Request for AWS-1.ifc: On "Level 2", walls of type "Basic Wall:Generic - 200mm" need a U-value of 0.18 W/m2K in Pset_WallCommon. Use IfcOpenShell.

First a look at what the model holds.

```python
import ifcopenshell
import ifcopenshell.util.element

model = ifcopenshell.open("AWS-1.ifc")
print(model.schema)
storey = next(s for s in model.by_type("IfcBuildingStorey") if s.Name == "Level 2")
walls = [e for e in ifcopenshell.util.element.get_decomposition(storey) if e.is_a("IfcWall")]
seen = {}
for e in walls:
    element_type = ifcopenshell.util.element.get_type(e)
    key = (element_type.Name if element_type != e and element_type else None, ifcopenshell.util.element.get_pset(e, "Pset_WallCommon", "ThermalTransmittance"))
    seen[key] = seen.get(key, 0) + 1
for (name, value), count in sorted(seen.items(), key=str):
    print(count, "x", name, "|", value)
```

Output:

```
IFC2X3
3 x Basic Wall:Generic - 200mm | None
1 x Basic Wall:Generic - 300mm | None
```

```python
import ifcopenshell
import ifcopenshell.api.pset
import ifcopenshell.util.element

model = ifcopenshell.open("AWS-1.ifc")

storey = next(s for s in model.by_type("IfcBuildingStorey") if s.Name == "Level 2")
walls = [e for e in ifcopenshell.util.element.get_decomposition(storey) if e.is_a("IfcWall")]

count = 0
for e in walls:
    element_type = ifcopenshell.util.element.get_type(e)
    if element_type in (None, e) or element_type.Name != "Basic Wall:Generic - 200mm":
        continue
    # add_pset returns the element's existing set when there is one.
    pset = ifcopenshell.api.pset.add_pset(model, product=e, name="Pset_WallCommon")
    ifcopenshell.api.pset.edit_pset(model, pset=pset, properties={"ThermalTransmittance": 0.18})
    count += 1

print(count, "walls updated")

model.write("AWS-1_rev.ifc")
```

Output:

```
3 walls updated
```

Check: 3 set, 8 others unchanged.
